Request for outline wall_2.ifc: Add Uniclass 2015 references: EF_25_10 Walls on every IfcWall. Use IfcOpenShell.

First a look at what the model holds.

```python
import ifcopenshell

model = ifcopenshell.open("outline wall_2.ifc")
print(model.schema)
print("classifications:", [c.Name for c in model.by_type("IfcClassification")])
for ifc_class in ("IfcDoor", "IfcRoof", "IfcStair", "IfcWall", "IfcWindow"):
    print(ifc_class, len(model.by_type(ifc_class)))
```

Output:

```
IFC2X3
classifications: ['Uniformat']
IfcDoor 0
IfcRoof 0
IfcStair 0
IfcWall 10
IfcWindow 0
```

```python
import ifcopenshell
import ifcopenshell.api.classification

model = ifcopenshell.open("outline wall_2.ifc")

# IFC2X3 requires Source and Edition and has no link from the project to the system.
system = model.create_entity("IfcClassification", Source="NBS", Edition="2015", Name="Uniclass 2015")

codes = {
    "IfcWall": ("EF_25_10", "Walls"),
}
for ifc_class, (code, name) in codes.items():
    products = model.by_type(ifc_class)
    ifcopenshell.api.classification.add_reference(
        model, products=products, classification=system, identification=code, name=name
    )
    print(code, len(products))

model.write("outline wall_2_updated.ifc")
```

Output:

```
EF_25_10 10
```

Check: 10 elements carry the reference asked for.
